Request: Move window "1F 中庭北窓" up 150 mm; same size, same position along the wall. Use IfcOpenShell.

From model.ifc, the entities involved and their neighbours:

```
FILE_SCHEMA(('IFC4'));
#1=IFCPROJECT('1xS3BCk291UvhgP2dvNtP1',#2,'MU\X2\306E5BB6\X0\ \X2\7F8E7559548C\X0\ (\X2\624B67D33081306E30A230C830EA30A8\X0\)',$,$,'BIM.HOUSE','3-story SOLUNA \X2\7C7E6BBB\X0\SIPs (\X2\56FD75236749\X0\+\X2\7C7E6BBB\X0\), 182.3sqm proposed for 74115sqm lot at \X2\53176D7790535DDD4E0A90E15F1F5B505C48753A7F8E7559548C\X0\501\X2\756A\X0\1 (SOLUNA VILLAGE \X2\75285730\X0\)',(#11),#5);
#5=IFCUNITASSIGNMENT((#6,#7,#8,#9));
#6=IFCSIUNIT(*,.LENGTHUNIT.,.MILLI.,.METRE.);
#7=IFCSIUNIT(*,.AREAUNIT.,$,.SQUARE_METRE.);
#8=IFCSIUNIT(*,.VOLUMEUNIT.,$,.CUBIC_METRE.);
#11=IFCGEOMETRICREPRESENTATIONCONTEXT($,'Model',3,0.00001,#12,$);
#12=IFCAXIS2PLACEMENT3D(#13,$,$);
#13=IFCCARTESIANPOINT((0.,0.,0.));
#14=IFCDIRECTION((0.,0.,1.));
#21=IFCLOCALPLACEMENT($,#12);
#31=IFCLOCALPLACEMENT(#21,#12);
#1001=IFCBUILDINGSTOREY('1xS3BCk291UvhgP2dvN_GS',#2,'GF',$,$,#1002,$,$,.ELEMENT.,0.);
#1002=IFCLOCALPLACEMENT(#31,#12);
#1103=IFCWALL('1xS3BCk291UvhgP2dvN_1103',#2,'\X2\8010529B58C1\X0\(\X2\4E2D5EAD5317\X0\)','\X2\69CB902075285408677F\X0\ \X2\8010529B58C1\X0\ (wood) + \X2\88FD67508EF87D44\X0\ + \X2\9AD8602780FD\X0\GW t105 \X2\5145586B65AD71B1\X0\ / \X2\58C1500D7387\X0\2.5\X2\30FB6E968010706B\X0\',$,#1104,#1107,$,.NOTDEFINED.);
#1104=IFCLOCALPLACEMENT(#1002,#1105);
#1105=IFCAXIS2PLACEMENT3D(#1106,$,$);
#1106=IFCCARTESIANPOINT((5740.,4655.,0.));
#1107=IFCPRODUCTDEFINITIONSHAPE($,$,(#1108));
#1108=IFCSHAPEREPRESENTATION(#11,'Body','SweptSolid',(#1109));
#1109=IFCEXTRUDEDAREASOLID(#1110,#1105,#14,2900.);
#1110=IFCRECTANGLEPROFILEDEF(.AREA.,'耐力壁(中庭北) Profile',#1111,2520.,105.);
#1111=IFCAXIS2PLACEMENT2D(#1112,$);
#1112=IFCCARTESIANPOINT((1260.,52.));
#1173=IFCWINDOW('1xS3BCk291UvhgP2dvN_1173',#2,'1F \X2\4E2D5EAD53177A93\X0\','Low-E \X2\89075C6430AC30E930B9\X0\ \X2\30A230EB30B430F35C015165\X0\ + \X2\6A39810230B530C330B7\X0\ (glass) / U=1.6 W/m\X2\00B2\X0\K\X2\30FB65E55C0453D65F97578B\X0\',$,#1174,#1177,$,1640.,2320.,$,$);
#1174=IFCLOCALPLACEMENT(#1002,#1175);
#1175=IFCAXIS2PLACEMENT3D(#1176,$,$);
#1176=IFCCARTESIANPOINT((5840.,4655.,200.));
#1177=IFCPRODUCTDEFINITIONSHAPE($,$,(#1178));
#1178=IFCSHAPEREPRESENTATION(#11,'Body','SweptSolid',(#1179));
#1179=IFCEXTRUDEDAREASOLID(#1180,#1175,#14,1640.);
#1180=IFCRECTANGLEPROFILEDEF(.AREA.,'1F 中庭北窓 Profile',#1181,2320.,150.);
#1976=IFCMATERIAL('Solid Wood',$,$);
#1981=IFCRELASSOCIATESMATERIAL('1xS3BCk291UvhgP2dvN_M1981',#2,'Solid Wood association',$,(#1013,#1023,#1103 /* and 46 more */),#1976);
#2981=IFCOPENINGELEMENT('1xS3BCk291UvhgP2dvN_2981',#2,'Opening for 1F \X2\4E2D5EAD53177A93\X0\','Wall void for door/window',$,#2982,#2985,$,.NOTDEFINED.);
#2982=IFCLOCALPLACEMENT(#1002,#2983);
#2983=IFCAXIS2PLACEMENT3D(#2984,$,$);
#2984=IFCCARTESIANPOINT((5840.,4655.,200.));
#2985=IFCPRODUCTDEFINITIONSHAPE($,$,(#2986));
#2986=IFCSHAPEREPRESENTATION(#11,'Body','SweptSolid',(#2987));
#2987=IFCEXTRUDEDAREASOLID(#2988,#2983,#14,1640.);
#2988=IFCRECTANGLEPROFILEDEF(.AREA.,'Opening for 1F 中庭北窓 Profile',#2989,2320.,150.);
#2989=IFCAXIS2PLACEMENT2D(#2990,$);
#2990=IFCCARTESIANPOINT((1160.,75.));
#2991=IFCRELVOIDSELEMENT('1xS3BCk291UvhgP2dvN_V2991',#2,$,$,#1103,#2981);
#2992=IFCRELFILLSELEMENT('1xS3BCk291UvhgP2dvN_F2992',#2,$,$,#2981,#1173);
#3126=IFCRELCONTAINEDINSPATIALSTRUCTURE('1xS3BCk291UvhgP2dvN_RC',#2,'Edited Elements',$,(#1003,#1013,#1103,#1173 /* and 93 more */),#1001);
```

```python
import numpy as np
import ifcopenshell
import ifcopenshell.api.geometry
import ifcopenshell.util.placement
import ifcopenshell.util.unit

model = ifcopenshell.open("model.ifc")
unit_scale = ifcopenshell.util.unit.calculate_unit_scale(model)

window = model.by_guid("1xS3BCk291UvhgP2dvN_1173")
opening = window.FillsVoids[0].RelatingOpeningElement
dz = 0.15 / unit_scale

shift = np.array([0.0, 0.0, dz])
# The window is not placed relative to its opening, so move both.
for product in (opening, window):
    matrix = ifcopenshell.util.placement.get_local_placement(product.ObjectPlacement)
    matrix[:3, 3] += shift
    ifcopenshell.api.geometry.edit_object_placement(model, product=product, matrix=matrix, is_si=False)

print(f"moved by {dz * unit_scale:+.3f} m")

model.write("model_rev.ifc")
```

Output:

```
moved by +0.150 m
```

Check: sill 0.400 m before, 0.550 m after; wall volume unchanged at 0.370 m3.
